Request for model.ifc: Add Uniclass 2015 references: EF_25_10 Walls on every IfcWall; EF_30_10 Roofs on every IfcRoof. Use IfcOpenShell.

First a look at what the model holds.

```python
import ifcopenshell

model = ifcopenshell.open("model.ifc")
print(model.schema)
print("classifications:", [c.Name for c in model.by_type("IfcClassification")])
for ifc_class in ("IfcDoor", "IfcRoof", "IfcStair", "IfcWall", "IfcWindow"):
    print(ifc_class, len(model.by_type(ifc_class)))
```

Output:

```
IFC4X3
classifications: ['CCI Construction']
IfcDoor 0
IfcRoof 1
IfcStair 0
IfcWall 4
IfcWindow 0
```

```python
import ifcopenshell
import ifcopenshell.api.classification

model = ifcopenshell.open("model.ifc")

system = ifcopenshell.api.classification.add_classification(model, classification="Uniclass 2015")

codes = {
    "IfcWall": ("EF_25_10", "Walls"),
    "IfcRoof": ("EF_30_10", "Roofs"),
}
for ifc_class, (code, name) in codes.items():
    products = model.by_type(ifc_class)
    ifcopenshell.api.classification.add_reference(
        model, products=products, classification=system, identification=code, name=name
    )
    print(code, len(products))

model.write("model_edited.ifc")
```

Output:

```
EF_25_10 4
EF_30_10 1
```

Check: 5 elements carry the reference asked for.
